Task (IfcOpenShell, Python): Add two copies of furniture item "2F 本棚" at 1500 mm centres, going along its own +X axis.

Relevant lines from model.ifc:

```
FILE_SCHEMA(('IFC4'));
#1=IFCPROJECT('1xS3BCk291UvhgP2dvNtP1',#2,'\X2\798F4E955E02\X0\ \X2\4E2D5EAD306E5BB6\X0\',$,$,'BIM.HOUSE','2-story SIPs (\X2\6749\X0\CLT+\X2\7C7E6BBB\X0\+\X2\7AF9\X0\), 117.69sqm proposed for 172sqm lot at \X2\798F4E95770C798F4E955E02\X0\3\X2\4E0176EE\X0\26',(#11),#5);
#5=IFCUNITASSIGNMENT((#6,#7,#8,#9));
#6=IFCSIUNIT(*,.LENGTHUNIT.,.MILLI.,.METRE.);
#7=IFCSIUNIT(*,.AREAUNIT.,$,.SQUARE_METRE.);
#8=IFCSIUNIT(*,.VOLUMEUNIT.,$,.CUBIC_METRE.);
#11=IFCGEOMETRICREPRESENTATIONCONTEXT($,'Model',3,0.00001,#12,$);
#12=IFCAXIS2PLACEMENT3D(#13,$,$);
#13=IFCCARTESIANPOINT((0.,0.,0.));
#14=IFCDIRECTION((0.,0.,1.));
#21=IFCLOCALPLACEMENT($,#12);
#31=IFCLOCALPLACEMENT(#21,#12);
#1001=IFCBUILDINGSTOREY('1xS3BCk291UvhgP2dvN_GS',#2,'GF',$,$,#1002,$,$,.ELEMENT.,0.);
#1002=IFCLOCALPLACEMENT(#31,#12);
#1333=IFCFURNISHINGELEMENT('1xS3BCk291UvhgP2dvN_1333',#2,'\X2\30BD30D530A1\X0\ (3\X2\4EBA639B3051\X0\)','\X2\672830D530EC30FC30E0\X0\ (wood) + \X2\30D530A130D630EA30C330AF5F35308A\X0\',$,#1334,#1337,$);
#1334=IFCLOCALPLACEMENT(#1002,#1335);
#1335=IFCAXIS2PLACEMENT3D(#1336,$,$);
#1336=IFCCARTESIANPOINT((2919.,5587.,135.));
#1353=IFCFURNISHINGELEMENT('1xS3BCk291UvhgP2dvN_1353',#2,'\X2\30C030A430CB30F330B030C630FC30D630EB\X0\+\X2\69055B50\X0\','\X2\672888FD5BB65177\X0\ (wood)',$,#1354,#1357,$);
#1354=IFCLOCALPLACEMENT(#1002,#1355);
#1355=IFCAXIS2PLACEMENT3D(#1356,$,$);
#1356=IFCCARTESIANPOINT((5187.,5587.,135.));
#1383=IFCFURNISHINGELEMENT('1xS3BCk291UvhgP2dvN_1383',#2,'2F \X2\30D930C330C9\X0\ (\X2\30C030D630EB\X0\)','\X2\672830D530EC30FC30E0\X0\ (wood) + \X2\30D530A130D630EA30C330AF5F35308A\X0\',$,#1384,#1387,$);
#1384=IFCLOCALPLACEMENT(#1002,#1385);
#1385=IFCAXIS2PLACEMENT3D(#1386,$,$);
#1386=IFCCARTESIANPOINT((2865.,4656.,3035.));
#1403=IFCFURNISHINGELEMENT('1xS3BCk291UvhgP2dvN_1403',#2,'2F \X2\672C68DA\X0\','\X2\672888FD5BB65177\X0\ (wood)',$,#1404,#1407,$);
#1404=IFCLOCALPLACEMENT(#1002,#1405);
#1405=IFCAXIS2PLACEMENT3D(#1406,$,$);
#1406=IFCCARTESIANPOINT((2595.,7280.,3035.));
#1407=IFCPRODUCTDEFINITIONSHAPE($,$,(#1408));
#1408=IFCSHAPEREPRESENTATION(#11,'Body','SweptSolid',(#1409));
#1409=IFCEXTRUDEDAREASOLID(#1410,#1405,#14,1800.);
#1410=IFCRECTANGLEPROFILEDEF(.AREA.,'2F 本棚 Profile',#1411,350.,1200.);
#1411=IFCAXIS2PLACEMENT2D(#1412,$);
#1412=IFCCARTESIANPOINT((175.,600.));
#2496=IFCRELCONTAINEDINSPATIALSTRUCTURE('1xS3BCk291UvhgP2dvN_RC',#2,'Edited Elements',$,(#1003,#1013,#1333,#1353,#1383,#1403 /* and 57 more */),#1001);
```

```python
import ifcopenshell
import ifcopenshell.api.geometry
import ifcopenshell.api.root
import ifcopenshell.util.element
import ifcopenshell.util.placement

model = ifcopenshell.open("model.ifc")


def reuse_history(source, copy):
    """copy_class also copies each property set's owner history, people and application; keep the originals."""
    for rel in copy.IsDefinedBy:
        if rel.is_a("IfcRelDefinesByProperties") and (history := rel.RelatingPropertyDefinition.OwnerHistory):
            rel.RelatingPropertyDefinition.OwnerHistory = source.OwnerHistory
            ifcopenshell.util.element.remove_deep2(model, history)


source = model.by_id(1403)
base = ifcopenshell.util.placement.get_local_placement(source.ObjectPlacement)
step = base[:3, 0] * 1500.0

for i in range(1, 3):
    copy = ifcopenshell.api.root.copy_class(model, product=source)
    copy.Representation = ifcopenshell.util.element.copy_deep(
        model, source.Representation, exclude=["IfcGeometricRepresentationContext", "IfcRepresentationMap"]
    )
    reuse_history(source, copy)
    matrix = base.copy()
    matrix[:3, 3] += i * step
    print("added at", matrix[:3, 3].round(3) + 0.0)
    ifcopenshell.api.geometry.edit_object_placement(model, product=copy, matrix=matrix, is_si=False)

model.write("model-out.ifc")
```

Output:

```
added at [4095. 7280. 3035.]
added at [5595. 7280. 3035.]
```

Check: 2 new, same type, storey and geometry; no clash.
